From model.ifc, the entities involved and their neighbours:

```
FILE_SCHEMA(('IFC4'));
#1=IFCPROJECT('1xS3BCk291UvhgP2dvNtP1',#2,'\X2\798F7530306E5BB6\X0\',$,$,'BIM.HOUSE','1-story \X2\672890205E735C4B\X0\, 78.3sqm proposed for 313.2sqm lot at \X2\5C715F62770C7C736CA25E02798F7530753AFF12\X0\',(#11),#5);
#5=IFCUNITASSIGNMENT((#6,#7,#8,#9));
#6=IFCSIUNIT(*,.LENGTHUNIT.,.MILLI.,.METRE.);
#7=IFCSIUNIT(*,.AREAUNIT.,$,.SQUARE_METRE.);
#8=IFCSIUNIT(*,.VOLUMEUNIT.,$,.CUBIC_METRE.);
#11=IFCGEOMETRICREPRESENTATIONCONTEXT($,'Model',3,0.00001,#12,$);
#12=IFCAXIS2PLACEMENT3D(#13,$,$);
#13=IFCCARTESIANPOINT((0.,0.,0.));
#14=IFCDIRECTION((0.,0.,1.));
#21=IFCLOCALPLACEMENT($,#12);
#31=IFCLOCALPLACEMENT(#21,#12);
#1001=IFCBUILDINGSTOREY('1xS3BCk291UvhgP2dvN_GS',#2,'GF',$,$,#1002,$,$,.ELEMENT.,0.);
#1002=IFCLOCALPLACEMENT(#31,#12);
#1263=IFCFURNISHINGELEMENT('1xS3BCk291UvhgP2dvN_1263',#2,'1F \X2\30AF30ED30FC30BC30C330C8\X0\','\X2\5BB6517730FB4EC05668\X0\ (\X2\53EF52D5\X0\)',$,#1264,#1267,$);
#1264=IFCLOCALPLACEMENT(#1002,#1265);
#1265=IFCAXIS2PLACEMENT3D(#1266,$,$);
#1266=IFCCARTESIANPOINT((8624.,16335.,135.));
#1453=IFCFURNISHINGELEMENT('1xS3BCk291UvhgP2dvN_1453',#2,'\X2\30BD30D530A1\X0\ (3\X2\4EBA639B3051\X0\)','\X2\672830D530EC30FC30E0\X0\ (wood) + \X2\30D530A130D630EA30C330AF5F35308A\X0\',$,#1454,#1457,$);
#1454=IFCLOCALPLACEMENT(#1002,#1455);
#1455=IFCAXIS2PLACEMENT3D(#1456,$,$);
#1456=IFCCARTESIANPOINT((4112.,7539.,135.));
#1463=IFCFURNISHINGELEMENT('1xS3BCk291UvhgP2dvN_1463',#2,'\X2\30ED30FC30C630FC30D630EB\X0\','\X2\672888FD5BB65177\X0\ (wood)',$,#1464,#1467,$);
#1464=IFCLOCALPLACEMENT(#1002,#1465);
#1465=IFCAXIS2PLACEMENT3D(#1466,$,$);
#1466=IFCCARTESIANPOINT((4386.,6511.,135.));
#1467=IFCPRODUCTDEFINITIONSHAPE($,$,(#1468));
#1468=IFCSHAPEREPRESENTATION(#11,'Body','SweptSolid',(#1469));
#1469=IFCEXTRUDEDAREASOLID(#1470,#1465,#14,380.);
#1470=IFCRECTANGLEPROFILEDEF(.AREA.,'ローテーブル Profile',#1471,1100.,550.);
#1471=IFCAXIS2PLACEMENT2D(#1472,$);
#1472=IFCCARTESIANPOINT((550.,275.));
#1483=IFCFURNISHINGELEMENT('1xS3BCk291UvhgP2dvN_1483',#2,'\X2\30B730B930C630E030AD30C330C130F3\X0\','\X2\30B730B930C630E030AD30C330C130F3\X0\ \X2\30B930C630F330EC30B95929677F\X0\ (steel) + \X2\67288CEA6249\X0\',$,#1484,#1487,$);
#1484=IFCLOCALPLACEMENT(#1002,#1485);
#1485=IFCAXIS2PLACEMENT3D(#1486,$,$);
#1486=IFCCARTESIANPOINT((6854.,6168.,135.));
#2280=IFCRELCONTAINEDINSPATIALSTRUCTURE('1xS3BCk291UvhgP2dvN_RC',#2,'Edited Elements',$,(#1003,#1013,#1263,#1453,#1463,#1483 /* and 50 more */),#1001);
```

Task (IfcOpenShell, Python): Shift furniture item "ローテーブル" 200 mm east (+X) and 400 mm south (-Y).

```python
import ifcopenshell
import ifcopenshell.api.geometry
import ifcopenshell.util.placement
import ifcopenshell.util.unit

model = ifcopenshell.open("model.ifc")
unit_scale = ifcopenshell.util.unit.calculate_unit_scale(model)

item = model.by_guid("1xS3BCk291UvhgP2dvN_1463")
matrix = ifcopenshell.util.placement.get_local_placement(item.ObjectPlacement)
matrix[0, 3] += 0.2 / unit_scale
matrix[1, 3] -= 0.4 / unit_scale
ifcopenshell.api.geometry.edit_object_placement(model, product=item, matrix=matrix, is_si=False)

print(ifcopenshell.util.placement.get_local_placement(item.ObjectPlacement).round(3) + 0.0)

model.write("model_updated.ifc")
```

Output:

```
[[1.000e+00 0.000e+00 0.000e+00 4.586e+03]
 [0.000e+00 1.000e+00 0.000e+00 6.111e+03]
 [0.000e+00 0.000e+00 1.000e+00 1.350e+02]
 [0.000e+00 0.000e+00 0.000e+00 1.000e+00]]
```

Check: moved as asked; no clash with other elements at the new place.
